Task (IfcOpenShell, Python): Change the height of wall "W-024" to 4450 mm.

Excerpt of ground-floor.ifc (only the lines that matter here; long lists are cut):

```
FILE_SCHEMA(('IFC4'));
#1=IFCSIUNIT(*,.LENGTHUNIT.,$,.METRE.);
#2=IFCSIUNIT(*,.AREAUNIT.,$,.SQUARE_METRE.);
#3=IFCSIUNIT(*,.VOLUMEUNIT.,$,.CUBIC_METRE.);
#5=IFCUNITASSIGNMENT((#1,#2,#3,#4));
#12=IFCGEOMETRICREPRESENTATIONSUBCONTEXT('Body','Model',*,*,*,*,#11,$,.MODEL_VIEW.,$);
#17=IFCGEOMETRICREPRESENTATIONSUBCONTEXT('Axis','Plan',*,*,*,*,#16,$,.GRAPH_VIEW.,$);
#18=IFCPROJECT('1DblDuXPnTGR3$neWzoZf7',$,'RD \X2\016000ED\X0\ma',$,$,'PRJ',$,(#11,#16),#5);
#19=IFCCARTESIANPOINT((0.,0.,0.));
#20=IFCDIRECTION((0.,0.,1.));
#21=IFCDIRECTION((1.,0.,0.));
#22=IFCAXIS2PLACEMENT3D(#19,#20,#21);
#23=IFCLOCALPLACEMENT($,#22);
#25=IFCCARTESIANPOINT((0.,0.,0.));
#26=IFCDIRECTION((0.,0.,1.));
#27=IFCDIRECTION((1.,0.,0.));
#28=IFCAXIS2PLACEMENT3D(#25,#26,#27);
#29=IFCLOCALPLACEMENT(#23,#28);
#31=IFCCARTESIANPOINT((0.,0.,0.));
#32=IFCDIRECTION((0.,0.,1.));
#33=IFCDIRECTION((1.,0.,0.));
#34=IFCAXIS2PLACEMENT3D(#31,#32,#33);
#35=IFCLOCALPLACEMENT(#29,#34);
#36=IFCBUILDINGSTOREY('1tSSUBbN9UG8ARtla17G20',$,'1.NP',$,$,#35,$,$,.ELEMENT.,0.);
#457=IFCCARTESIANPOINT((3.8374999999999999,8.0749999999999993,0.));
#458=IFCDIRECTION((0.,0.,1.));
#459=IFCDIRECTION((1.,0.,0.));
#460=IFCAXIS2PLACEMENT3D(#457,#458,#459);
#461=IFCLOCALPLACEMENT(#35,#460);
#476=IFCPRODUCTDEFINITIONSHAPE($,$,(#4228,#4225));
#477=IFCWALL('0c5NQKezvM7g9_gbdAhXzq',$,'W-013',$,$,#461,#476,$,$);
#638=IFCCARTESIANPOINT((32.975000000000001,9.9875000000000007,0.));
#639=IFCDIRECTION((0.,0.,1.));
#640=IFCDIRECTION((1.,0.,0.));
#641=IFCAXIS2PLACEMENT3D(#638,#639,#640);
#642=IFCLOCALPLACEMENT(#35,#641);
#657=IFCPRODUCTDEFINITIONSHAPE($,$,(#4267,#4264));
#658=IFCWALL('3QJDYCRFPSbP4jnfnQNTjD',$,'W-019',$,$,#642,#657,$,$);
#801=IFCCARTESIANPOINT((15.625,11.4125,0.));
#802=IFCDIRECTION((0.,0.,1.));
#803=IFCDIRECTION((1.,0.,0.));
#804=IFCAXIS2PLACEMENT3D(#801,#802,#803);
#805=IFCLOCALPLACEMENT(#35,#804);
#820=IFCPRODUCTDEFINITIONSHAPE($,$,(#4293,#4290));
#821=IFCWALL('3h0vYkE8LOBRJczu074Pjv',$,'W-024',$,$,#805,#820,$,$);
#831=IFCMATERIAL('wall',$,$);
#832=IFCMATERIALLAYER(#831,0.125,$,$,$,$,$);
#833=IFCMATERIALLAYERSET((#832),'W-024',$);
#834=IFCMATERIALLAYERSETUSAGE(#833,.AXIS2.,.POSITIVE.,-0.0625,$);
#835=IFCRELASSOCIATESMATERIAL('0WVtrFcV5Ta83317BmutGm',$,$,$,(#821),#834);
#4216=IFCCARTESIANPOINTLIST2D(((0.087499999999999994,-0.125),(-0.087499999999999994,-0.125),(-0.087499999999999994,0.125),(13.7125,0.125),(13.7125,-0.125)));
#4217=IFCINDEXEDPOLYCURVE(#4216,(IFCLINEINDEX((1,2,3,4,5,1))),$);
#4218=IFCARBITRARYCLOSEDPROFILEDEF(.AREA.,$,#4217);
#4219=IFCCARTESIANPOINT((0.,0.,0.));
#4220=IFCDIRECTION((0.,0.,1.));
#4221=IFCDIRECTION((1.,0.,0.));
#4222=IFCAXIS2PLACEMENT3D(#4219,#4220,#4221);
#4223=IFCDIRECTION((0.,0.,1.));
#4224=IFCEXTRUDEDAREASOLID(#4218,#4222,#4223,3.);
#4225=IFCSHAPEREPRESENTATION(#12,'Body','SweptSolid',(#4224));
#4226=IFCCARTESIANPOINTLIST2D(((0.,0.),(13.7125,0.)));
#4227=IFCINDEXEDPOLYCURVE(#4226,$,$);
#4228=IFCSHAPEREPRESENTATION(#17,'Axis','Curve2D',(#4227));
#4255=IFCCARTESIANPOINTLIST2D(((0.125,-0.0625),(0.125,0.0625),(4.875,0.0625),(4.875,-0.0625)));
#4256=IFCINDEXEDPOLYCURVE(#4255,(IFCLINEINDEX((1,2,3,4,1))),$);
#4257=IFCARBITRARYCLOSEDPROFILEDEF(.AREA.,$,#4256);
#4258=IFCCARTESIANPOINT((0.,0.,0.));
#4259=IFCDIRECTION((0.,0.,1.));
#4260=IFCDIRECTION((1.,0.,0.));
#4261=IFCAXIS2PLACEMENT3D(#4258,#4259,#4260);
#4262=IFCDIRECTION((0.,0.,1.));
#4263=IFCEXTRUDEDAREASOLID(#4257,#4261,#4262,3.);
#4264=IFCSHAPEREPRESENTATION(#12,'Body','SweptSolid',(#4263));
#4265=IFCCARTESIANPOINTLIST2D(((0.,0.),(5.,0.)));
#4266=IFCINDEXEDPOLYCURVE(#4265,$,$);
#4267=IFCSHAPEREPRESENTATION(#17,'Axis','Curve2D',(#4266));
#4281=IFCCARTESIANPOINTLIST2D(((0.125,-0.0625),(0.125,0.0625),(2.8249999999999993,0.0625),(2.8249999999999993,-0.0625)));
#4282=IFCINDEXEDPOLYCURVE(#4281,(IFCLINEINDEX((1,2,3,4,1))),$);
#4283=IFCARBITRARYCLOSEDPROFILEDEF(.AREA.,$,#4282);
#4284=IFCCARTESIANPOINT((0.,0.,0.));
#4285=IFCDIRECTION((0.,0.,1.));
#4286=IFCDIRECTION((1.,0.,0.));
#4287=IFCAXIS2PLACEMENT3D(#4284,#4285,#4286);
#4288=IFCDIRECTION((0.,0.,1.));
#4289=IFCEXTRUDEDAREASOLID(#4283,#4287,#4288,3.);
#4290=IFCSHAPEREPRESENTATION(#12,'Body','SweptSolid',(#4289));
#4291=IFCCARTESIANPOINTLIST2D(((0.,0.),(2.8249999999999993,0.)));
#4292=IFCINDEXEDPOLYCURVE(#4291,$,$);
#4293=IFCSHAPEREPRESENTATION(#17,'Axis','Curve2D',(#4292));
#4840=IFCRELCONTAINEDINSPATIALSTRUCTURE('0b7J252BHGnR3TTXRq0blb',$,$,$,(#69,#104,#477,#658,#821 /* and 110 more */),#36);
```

```python
import ifcopenshell
import ifcopenshell.geom
import ifcopenshell.util.representation
import ifcopenshell.util.shape

model = ifcopenshell.open("ground-floor.ifc")
settings = ifcopenshell.geom.settings()


def volume(element):
    """Net volume in cubic metres, openings subtracted."""
    shape = ifcopenshell.geom.create_shape(settings, element)
    return ifcopenshell.util.shape.get_volume(shape.geometry)


wall = model.by_guid("3h0vYkE8LOBRJczu074Pjv")
before = volume(wall)

body = ifcopenshell.util.representation.get_representation(wall, "Model", "Body")
solid = body.Items[0]
old_height = solid.Depth
solid.Depth = 4.45
after = volume(wall)

print(f"height {old_height:g} -> {solid.Depth:g}, volume {before:.3f} -> {after:.3f} m3")

model.write("ground-floor-out.ifc")
```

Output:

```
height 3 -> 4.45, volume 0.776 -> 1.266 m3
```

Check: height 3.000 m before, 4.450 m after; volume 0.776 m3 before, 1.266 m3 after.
